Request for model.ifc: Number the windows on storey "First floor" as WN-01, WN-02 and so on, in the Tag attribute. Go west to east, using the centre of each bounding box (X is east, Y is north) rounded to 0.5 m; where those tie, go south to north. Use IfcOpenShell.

First a look at what the model holds.

```python
import ifcopenshell
import ifcopenshell.util.element
import ifcopenshell.util.placement

model = ifcopenshell.open("model.ifc")
print(model.schema)
storey = next(s for s in model.by_type("IfcBuildingStorey") if s.Name == "First floor")
windows = [e for e in ifcopenshell.util.element.get_decomposition(storey) if e.is_a("IfcWindow")]
for e in sorted(windows, key=lambda e: e.id()):
    origin = ifcopenshell.util.placement.get_local_placement(e.ObjectPlacement)[:3, 3]
    print(e.id(), e.Tag, e.Name, origin.round(2) + 0.0, sep=" | ")
```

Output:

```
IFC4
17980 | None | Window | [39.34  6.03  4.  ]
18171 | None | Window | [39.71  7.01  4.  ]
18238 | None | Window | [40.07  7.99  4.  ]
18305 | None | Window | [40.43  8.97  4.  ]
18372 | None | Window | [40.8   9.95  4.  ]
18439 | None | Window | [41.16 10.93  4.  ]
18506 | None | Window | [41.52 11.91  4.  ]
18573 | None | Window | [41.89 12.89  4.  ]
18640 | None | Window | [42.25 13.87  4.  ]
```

```python
import ifcopenshell
import ifcopenshell.geom
import ifcopenshell.util.element
import ifcopenshell.util.shape

model = ifcopenshell.open("model.ifc")
settings = ifcopenshell.geom.settings()
settings.set("use-world-coords", True)


def centre(element):
    shape = ifcopenshell.geom.create_shape(settings, element)
    return ifcopenshell.util.shape.get_bbox_centroid(shape.geometry)


storey = next(s for s in model.by_type("IfcBuildingStorey") if s.Name == "First floor")
windows = [e for e in ifcopenshell.util.element.get_decomposition(storey) if e.is_a("IfcWindow")]

# Insertion points can sit at a corner or the storey origin, so sort by the geometry (in metres).
centres = {e: centre(e) for e in windows}
windows.sort(key=lambda e: (round(centres[e][0] / 0.5), centres[e][1]))

for i, e in enumerate(windows, start=1):
    number = f"WN-{i:02d}"
    e.Tag = number
    print(e.id(), number)

model.write("model_edited.ifc")
```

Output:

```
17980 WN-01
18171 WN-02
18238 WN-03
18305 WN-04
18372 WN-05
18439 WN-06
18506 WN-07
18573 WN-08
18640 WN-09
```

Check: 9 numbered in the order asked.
